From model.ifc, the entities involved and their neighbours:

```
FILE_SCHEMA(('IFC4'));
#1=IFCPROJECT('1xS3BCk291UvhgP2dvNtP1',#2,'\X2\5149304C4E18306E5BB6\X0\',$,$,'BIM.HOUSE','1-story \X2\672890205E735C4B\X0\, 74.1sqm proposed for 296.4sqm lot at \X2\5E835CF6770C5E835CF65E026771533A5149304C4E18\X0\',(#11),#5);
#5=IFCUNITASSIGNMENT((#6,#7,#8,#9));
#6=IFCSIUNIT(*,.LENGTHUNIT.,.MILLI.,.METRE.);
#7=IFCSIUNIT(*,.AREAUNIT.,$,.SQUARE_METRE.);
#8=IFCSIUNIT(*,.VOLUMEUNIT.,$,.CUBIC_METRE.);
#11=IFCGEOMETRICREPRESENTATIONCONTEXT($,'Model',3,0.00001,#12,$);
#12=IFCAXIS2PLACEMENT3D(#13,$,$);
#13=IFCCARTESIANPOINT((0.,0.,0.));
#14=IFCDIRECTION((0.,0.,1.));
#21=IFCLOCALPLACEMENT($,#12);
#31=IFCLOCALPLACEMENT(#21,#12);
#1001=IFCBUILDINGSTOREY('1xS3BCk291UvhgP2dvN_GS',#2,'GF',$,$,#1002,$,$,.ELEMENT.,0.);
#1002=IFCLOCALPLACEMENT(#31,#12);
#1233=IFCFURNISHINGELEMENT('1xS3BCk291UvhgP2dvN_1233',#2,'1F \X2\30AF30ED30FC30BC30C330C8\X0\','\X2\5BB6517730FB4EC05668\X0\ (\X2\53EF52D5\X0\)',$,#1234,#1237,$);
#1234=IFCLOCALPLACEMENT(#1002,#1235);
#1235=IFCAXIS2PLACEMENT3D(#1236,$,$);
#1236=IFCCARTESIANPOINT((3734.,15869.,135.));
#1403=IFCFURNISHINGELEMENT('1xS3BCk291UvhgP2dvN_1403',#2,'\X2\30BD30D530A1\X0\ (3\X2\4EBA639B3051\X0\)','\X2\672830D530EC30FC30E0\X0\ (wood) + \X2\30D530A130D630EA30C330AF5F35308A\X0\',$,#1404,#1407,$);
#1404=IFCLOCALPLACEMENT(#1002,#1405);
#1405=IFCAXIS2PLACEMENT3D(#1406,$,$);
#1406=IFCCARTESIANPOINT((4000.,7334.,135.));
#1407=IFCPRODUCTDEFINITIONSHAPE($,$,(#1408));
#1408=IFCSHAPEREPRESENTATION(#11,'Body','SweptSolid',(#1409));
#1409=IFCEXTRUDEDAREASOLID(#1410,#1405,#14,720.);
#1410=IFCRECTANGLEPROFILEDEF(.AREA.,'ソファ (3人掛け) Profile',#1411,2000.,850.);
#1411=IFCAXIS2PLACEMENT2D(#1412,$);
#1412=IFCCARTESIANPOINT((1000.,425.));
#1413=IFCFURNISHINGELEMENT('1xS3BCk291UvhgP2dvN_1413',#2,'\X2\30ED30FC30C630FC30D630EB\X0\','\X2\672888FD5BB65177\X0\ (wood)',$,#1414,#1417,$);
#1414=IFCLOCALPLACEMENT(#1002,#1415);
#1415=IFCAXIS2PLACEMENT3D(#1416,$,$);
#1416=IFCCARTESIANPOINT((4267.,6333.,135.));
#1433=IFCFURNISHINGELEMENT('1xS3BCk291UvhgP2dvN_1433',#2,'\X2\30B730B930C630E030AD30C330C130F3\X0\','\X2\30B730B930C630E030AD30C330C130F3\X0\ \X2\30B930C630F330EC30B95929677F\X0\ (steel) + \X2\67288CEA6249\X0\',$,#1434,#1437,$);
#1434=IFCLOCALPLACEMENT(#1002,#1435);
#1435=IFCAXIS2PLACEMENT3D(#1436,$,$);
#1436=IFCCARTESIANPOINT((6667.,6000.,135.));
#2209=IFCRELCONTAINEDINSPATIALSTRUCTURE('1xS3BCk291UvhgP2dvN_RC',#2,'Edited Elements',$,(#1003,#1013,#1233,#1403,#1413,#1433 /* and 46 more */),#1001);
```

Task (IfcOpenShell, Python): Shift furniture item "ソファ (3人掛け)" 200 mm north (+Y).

```python
import ifcopenshell
import ifcopenshell.api.geometry
import ifcopenshell.util.placement
import ifcopenshell.util.unit

model = ifcopenshell.open("model.ifc")
unit_scale = ifcopenshell.util.unit.calculate_unit_scale(model)

item = model.by_id(1403)
matrix = ifcopenshell.util.placement.get_local_placement(item.ObjectPlacement)
matrix[1, 3] += 0.2 / unit_scale
ifcopenshell.api.geometry.edit_object_placement(model, product=item, matrix=matrix, is_si=False)

print(ifcopenshell.util.placement.get_local_placement(item.ObjectPlacement).round(3) + 0.0)

model.write("model_rev.ifc")
```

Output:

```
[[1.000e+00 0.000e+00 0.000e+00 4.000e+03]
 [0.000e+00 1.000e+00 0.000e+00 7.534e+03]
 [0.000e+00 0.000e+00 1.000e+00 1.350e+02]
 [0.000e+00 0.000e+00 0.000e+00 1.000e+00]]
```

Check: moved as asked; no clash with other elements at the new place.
